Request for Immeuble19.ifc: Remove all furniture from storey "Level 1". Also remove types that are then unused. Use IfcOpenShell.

First a look at what the model holds.

```python
import ifcopenshell
import ifcopenshell.util.element

model = ifcopenshell.open("Immeuble19.ifc")
print(model.schema)
storey = next(s for s in model.by_type("IfcBuildingStorey") if s.Name == "Level 1")
furniture = [e for e in ifcopenshell.util.element.get_decomposition(storey) if e.is_a("IfcFurnishingElement")]
seen = {}
for e in furniture:
    element_type = ifcopenshell.util.element.get_type(e)
    name = element_type.Name if element_type not in (None, e) else None
    seen[name] = seen.get(name, 0) + 1
for name, count in sorted(seen.items(), key=str):
    print(count, "x", name)
```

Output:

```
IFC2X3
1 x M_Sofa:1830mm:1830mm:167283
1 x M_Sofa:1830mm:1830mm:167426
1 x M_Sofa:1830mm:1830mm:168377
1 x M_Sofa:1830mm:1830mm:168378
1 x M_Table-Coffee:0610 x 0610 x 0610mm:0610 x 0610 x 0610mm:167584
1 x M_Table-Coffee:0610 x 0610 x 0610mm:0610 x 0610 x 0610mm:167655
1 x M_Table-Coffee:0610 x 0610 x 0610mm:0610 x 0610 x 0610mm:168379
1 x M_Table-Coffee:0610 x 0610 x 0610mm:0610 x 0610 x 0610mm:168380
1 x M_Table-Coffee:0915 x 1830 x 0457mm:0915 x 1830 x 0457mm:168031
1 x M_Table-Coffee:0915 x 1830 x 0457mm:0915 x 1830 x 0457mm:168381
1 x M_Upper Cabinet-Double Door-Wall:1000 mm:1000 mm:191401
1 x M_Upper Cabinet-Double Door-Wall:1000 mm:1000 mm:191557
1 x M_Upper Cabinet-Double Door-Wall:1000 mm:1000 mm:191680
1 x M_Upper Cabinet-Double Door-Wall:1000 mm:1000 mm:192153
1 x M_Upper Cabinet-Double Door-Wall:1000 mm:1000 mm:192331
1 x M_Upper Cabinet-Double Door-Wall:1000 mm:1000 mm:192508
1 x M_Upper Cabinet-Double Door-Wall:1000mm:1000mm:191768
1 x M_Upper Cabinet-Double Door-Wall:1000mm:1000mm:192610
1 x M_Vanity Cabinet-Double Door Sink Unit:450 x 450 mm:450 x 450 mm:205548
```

```python
import ifcopenshell
import ifcopenshell.api.root
import ifcopenshell.util.element

model = ifcopenshell.open("Immeuble19.ifc")

storey = next(s for s in model.by_type("IfcBuildingStorey") if s.Name == "Level 1")
furniture = [e for e in ifcopenshell.util.element.get_decomposition(storey) if e.is_a("IfcFurnishingElement")]
types = {ifcopenshell.util.element.get_type(e) for e in furniture} - {None, *furniture}

for e in furniture:
    ifcopenshell.api.root.remove_product(model, product=e)
print(len(furniture), "removed")

unused = [t for t in types if not ifcopenshell.util.element.get_types(t)]
for t in unused:
    ifcopenshell.api.root.remove_product(model, product=t)
print(len(unused), "unused types removed")

model.write("Immeuble19-out.ifc")
```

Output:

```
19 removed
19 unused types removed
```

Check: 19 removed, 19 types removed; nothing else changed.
